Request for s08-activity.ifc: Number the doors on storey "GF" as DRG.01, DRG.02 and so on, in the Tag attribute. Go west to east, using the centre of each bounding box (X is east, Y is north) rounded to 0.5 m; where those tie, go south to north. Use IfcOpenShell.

First a look at what the model holds.

```python
import ifcopenshell
import ifcopenshell.util.element
import ifcopenshell.util.placement

model = ifcopenshell.open("s08-activity.ifc")
print(model.schema)
storey = next(s for s in model.by_type("IfcBuildingStorey") if s.Name == "GF")
doors = [e for e in ifcopenshell.util.element.get_decomposition(storey) if e.is_a("IfcDoor")]
for e in sorted(doors, key=lambda e: e.id()):
    origin = ifcopenshell.util.placement.get_local_placement(e.ObjectPlacement)[:3, 3]
    print(e.id(), e.Tag, e.Name, origin.round(2) + 0.0, sep=" | ")
```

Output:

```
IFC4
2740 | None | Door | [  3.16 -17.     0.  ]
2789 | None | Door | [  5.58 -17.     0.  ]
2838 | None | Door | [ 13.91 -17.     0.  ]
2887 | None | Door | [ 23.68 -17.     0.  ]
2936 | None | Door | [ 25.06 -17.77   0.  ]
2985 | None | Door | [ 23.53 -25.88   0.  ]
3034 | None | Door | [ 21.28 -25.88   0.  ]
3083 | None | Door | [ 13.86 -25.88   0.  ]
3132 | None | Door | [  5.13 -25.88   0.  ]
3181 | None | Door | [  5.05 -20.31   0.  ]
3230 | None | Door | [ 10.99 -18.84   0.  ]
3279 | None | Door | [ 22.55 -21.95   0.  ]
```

```python
import ifcopenshell
import ifcopenshell.geom
import ifcopenshell.util.element
import ifcopenshell.util.shape

model = ifcopenshell.open("s08-activity.ifc")
settings = ifcopenshell.geom.settings()
settings.set("use-world-coords", True)


def centre(element):
    shape = ifcopenshell.geom.create_shape(settings, element)
    return ifcopenshell.util.shape.get_bbox_centroid(shape.geometry)


storey = next(s for s in model.by_type("IfcBuildingStorey") if s.Name == "GF")
doors = [e for e in ifcopenshell.util.element.get_decomposition(storey) if e.is_a("IfcDoor")]

# Insertion points can sit at a corner or the storey origin, so sort by the geometry (in metres).
centres = {e: centre(e) for e in doors}
doors.sort(key=lambda e: (round(centres[e][0] / 0.5), centres[e][1]))

for i, e in enumerate(doors, start=1):
    number = f"DRG.{i:02d}"
    e.Tag = number
    print(e.id(), number)

model.write("s08-activity-out.ifc")
```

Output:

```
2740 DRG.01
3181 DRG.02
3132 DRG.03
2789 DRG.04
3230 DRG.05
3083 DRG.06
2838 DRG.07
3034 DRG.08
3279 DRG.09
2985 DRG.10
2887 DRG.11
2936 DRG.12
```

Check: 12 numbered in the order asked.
